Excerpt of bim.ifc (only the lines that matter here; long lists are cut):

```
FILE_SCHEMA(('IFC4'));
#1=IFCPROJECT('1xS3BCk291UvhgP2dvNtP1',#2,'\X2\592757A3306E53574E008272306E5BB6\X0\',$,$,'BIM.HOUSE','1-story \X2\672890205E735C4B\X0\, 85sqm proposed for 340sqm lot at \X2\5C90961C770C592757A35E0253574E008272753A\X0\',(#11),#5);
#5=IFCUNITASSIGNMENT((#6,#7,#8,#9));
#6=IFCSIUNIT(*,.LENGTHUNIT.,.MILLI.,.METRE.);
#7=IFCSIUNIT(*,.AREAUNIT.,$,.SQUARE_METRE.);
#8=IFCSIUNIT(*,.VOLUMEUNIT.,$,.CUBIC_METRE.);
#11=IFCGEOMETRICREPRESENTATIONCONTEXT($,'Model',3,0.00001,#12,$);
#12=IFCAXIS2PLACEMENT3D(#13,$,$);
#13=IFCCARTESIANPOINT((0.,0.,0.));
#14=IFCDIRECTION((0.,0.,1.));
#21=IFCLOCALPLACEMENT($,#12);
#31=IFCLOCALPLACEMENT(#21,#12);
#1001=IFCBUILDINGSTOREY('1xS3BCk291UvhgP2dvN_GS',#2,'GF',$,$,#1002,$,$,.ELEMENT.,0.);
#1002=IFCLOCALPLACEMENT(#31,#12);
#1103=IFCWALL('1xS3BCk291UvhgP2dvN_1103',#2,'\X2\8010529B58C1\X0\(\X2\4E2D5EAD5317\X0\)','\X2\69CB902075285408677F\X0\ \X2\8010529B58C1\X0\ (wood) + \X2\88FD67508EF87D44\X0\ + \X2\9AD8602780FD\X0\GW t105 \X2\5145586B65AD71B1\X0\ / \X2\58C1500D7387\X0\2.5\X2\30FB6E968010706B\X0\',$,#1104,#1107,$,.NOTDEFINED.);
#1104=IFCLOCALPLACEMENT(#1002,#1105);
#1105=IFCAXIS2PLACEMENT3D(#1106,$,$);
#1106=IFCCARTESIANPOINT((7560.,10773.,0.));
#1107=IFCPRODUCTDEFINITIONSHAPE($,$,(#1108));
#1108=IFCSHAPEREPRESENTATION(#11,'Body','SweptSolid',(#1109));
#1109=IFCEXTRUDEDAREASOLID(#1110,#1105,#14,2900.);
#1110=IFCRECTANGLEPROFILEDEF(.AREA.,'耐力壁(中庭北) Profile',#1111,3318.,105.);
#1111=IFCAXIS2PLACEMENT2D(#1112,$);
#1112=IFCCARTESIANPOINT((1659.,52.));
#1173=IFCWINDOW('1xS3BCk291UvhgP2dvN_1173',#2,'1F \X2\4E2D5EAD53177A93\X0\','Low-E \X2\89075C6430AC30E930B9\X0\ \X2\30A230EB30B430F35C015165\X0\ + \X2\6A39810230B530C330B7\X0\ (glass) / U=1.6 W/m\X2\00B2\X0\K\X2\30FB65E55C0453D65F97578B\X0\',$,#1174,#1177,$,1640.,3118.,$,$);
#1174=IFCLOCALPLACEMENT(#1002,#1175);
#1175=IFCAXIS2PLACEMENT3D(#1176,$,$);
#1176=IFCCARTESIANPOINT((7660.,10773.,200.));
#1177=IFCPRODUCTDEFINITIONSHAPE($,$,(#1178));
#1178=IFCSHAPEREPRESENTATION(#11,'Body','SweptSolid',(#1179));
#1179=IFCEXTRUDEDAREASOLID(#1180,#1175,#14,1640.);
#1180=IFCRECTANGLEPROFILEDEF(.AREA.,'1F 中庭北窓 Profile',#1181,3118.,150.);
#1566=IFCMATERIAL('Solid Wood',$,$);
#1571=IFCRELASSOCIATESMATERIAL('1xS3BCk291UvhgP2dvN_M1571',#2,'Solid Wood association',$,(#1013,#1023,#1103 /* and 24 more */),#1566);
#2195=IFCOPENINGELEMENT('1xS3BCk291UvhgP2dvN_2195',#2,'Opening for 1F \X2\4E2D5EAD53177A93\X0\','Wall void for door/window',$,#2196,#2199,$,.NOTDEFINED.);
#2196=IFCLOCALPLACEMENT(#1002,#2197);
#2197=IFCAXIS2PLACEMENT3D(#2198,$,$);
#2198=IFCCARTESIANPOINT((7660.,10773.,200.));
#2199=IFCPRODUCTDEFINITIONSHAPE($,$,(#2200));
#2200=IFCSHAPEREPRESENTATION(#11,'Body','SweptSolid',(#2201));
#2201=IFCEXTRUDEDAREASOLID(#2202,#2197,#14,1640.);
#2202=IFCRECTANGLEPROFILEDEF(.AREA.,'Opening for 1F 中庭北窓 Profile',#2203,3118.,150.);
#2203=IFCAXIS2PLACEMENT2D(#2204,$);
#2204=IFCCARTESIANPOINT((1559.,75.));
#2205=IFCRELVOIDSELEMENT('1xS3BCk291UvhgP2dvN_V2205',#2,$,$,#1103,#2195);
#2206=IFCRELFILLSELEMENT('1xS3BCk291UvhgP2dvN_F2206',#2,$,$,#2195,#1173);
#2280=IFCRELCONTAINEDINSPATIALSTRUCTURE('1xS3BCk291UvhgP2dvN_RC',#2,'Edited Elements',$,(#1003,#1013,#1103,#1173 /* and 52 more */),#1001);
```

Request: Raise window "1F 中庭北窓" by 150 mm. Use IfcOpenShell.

```python
import numpy as np
import ifcopenshell
import ifcopenshell.api.geometry
import ifcopenshell.util.placement
import ifcopenshell.util.unit

model = ifcopenshell.open("bim.ifc")
unit_scale = ifcopenshell.util.unit.calculate_unit_scale(model)

window = model.by_id(1173)
opening = window.FillsVoids[0].RelatingOpeningElement
dz = 0.15 / unit_scale

shift = np.array([0.0, 0.0, dz])
# The window is not placed relative to its opening, so move both.
for product in (opening, window):
    matrix = ifcopenshell.util.placement.get_local_placement(product.ObjectPlacement)
    matrix[:3, 3] += shift
    ifcopenshell.api.geometry.edit_object_placement(model, product=product, matrix=matrix, is_si=False)

print(f"moved by {dz * unit_scale:+.3f} m")

model.write("bim_edited.ifc")
```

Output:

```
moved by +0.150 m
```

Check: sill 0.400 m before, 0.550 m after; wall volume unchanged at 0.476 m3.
